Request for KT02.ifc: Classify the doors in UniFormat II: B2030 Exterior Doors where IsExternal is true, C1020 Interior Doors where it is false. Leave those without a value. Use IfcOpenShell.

First a look at what the model holds.

```python
import ifcopenshell
import ifcopenshell.util.element

model = ifcopenshell.open("KT02.ifc")
print(model.schema)
print("classifications:", [c.Name for c in model.by_type("IfcClassification")])
values = [ifcopenshell.util.element.get_pset(e, "Pset_DoorCommon", "IsExternal") for e in model.by_type("IfcDoor")]
for value in (True, False, None):
    print("IsExternal", value, values.count(value))
```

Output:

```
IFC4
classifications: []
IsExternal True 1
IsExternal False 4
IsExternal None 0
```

```python
import ifcopenshell
import ifcopenshell.api.classification
import ifcopenshell.util.element

model = ifcopenshell.open("KT02.ifc")

system = ifcopenshell.api.classification.add_classification(model, classification="UniFormat II")

doors = model.by_type("IfcDoor")
external = {e: ifcopenshell.util.element.get_pset(e, "Pset_DoorCommon", "IsExternal") for e in doors}
for flag, code, name in ((True, "B2030", "Exterior Doors"), (False, "C1020", "Interior Doors")):
    products = [e for e in doors if external[e] is flag]
    ifcopenshell.api.classification.add_reference(
        model, products=products, classification=system, identification=code, name=name
    )
    print(code, len(products))

model.write("KT02_v2.ifc")
```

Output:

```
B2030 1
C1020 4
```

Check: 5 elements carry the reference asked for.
